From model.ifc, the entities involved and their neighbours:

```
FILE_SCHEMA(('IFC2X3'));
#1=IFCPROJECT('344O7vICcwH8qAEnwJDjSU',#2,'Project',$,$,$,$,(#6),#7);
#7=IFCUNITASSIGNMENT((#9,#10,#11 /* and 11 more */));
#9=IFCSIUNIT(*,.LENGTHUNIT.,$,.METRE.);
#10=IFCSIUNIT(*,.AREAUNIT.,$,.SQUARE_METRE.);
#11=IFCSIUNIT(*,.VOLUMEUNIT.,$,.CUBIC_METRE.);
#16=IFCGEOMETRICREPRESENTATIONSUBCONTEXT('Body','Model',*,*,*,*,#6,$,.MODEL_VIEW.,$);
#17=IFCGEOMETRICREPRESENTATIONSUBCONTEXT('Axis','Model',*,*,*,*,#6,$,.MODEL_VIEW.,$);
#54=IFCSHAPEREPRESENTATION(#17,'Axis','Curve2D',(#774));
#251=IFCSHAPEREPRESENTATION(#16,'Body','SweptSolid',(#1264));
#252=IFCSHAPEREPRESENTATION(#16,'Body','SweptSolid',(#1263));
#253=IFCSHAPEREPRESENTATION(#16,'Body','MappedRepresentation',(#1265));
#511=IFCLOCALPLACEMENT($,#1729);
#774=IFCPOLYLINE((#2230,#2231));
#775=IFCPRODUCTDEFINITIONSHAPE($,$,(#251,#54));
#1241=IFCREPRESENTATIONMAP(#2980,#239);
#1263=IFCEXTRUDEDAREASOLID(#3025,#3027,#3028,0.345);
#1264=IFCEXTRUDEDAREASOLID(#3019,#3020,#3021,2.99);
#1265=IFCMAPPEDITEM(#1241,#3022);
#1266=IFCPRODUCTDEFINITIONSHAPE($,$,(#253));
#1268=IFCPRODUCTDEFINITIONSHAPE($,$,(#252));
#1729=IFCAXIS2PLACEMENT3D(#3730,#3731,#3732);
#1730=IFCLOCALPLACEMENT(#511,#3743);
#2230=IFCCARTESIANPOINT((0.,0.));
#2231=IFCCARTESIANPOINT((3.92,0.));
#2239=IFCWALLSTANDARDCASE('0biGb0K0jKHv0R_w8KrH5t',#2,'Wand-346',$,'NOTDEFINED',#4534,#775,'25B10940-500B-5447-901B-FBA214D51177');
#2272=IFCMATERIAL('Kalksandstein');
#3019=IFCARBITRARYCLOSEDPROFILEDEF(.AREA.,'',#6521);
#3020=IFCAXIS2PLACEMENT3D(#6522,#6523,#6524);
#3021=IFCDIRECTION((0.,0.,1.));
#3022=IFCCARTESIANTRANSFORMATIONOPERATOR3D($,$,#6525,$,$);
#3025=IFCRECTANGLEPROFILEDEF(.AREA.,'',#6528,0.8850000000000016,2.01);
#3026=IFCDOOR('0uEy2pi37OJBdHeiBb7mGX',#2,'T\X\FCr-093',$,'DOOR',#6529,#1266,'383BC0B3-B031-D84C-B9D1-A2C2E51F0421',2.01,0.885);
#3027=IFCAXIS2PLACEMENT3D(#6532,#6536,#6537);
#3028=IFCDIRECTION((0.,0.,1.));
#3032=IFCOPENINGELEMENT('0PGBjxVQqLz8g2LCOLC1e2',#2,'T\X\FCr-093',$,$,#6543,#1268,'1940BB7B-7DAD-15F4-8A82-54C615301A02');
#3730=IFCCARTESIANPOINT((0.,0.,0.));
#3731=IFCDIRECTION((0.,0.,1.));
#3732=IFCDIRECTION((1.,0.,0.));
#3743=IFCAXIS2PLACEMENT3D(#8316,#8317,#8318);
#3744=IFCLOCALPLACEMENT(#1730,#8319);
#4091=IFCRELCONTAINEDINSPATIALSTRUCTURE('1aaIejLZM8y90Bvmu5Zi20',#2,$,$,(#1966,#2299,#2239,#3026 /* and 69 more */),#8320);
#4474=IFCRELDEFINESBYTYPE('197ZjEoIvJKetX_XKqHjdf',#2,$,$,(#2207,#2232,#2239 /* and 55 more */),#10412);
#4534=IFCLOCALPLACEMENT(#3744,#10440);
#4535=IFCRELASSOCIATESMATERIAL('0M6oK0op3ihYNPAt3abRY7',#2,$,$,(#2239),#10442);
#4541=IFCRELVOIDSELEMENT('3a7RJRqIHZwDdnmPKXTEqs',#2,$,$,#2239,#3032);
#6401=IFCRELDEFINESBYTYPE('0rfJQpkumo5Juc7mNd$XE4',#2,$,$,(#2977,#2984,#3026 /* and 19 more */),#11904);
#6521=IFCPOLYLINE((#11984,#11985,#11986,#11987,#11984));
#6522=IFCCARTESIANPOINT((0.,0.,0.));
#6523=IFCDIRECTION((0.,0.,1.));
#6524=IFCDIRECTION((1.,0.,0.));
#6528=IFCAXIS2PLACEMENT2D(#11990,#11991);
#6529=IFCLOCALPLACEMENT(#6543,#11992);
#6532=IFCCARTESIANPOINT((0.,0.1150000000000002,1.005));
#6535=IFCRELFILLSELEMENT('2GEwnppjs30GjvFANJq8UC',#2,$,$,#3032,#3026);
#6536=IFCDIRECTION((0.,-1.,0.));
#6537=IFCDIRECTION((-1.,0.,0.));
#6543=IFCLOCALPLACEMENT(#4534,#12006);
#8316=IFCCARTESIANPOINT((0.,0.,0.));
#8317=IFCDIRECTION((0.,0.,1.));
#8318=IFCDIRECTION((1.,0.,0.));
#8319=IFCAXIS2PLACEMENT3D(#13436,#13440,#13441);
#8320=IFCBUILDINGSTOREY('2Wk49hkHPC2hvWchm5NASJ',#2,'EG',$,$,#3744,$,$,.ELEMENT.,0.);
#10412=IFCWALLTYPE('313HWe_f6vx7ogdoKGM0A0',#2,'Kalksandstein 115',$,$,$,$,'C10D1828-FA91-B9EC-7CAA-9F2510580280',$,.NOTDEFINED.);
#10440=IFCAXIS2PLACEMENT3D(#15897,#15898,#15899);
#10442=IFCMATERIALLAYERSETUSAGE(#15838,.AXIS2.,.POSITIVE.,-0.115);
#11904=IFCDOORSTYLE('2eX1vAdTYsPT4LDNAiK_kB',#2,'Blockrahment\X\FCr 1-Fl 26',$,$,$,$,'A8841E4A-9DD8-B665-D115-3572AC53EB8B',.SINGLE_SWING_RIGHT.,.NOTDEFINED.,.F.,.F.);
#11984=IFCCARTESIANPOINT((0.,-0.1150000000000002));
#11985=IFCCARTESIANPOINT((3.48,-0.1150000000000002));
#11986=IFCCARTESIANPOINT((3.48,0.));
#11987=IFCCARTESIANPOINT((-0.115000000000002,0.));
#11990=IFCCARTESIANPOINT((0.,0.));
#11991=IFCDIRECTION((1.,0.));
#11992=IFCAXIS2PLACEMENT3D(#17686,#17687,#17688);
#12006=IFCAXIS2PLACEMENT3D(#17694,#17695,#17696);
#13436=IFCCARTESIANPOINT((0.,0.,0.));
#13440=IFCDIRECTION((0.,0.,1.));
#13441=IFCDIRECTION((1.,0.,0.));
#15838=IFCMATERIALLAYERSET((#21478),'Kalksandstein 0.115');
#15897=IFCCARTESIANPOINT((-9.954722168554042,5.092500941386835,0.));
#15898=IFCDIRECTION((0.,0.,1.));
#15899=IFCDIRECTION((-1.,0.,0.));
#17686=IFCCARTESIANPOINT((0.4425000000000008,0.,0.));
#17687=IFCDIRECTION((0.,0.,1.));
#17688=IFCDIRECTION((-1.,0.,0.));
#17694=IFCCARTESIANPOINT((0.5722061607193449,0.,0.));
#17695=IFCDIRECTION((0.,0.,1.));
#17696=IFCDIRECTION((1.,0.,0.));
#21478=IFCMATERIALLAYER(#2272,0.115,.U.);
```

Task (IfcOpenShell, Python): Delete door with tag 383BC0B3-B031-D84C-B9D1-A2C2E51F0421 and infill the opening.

```python
import ifcopenshell
import ifcopenshell.api.feature
import ifcopenshell.api.root
import ifcopenshell.geom
import ifcopenshell.util.shape

model = ifcopenshell.open("model.ifc")
settings = ifcopenshell.geom.settings()


def volume(element):
    """Net volume in cubic metres, openings subtracted."""
    shape = ifcopenshell.geom.create_shape(settings, element)
    return ifcopenshell.util.shape.get_volume(shape.geometry)


door = model.by_guid("0uEy2pi37OJBdHeiBb7mGX")
opening = door.FillsVoids[0].RelatingOpeningElement
wall = opening.VoidsElements[0].RelatingBuildingElement
before = volume(wall)

ifcopenshell.api.root.remove_product(model, product=door)
ifcopenshell.api.feature.remove_feature(model, feature=opening)

after = volume(wall)

print(f"wall volume {before:.3f} -> {after:.3f} m3")

model.write("model-out.ifc")
```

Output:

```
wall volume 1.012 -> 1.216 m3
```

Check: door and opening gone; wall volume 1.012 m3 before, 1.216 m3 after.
